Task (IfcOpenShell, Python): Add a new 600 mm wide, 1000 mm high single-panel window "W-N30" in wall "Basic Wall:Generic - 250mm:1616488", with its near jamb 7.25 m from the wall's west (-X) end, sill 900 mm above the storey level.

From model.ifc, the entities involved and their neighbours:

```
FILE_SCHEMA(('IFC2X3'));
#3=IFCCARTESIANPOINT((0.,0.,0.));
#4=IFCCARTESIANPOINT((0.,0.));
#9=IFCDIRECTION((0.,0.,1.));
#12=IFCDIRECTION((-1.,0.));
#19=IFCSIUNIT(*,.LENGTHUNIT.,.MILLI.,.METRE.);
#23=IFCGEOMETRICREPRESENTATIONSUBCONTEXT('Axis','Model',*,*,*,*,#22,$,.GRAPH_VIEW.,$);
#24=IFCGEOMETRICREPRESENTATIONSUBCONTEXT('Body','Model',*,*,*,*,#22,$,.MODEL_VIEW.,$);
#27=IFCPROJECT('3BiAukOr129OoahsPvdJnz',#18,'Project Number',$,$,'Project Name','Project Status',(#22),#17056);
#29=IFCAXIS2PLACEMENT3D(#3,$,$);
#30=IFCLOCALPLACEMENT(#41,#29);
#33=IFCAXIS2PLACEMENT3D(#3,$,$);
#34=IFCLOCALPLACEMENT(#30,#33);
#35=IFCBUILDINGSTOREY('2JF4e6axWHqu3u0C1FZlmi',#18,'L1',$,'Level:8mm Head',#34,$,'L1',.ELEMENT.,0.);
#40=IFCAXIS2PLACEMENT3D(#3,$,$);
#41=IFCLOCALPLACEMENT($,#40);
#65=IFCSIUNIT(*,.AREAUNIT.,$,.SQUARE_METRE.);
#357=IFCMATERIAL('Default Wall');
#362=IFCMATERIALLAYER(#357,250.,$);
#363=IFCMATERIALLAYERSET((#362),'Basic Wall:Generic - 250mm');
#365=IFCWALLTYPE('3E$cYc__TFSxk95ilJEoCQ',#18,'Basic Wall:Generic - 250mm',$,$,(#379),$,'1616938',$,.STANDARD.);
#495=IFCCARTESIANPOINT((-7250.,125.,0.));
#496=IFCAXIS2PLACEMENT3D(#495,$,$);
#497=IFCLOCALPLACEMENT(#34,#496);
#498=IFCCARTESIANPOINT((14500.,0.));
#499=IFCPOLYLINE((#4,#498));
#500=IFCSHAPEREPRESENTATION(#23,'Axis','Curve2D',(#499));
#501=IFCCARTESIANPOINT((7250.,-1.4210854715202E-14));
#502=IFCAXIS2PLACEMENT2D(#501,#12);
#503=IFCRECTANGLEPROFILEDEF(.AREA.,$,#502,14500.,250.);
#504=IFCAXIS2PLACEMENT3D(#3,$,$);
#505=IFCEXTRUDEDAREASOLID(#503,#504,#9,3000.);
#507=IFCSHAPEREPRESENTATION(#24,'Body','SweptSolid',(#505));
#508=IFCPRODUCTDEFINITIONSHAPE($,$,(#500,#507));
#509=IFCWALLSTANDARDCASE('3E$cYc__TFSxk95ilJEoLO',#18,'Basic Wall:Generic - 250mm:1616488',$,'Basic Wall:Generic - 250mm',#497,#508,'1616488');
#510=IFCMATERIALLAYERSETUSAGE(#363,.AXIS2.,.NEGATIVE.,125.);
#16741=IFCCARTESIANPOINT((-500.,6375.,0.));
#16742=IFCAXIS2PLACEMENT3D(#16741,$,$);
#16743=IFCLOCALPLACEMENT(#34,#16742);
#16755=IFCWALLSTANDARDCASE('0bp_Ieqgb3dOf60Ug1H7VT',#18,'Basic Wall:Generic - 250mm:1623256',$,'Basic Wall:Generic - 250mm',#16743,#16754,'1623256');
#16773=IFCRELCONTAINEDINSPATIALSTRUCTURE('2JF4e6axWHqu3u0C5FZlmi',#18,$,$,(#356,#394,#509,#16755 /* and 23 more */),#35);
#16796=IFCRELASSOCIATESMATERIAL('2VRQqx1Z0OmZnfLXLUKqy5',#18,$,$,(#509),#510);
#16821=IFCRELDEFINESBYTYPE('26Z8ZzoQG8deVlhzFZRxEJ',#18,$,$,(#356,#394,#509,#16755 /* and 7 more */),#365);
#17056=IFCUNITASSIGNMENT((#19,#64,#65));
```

```python
import numpy as np
import ifcopenshell
import ifcopenshell.api.feature
import ifcopenshell.api.geometry
import ifcopenshell.api.root
import ifcopenshell.api.spatial
import ifcopenshell.api.type
import ifcopenshell.geom
import ifcopenshell.util.element
import ifcopenshell.util.placement
import ifcopenshell.util.representation
import ifcopenshell.util.shape
import ifcopenshell.util.unit

model = ifcopenshell.open("model.ifc")
unit_scale = ifcopenshell.util.unit.calculate_unit_scale(model)
settings = ifcopenshell.geom.settings()


def volume(element):
    """Net volume in cubic metres, openings subtracted."""
    shape = ifcopenshell.geom.create_shape(settings, element)
    return ifcopenshell.util.shape.get_volume(shape.geometry)


wall = model.by_guid("3E$cYc__TFSxk95ilJEoLO")
storey = ifcopenshell.util.element.get_container(wall, ifc_class="IfcBuildingStorey")
context = ifcopenshell.util.representation.get_context(model, "Model", "Body", "MODEL_VIEW")
before = volume(wall)

width, height, from_end, sill = 0.6, 1, 7.25, 0.9  # metres

# The wall runs along its own X axis, and the end named is its -X end.
wall_shape = ifcopenshell.geom.create_shape(settings, wall)
x, y, z = ifcopenshell.util.shape.get_vertices(wall_shape.geometry).T
start = x.min() + from_end
face, thickness = float(y.min()), float(y.max() - y.min())
wall_matrix = ifcopenshell.util.placement.get_local_placement(wall.ObjectPlacement)
level = ifcopenshell.util.placement.get_local_placement(storey.ObjectPlacement)[2, 3]


def in_wall(x, y):
    """Placement at x, y metres in the wall's axes, at sill height."""
    matrix = wall_matrix.copy()
    matrix[:, 3] = wall_matrix @ np.array([x / unit_scale, y / unit_scale, 0.0, 1.0])
    matrix[2, 3] = level + sill / unit_scale
    return matrix


# Opening: a box that overshoots both wall faces by 50 mm.
opening = ifcopenshell.api.root.create_entity(model, ifc_class="IfcOpeningElement")
box = ifcopenshell.api.geometry.add_wall_representation(
    model, context=context, length=width, height=height, thickness=thickness + 0.1
)
ifcopenshell.api.geometry.assign_representation(model, product=opening, representation=box)
ifcopenshell.api.geometry.edit_object_placement(model, product=opening, matrix=in_wall(start, face - 0.05), is_si=False)
ifcopenshell.api.feature.add_feature(model, feature=opening, element=wall)

window = ifcopenshell.api.root.create_entity(model, ifc_class="IfcWindow", name="W-N30")
window.OverallWidth, window.OverallHeight = width / unit_scale, height / unit_scale
body = ifcopenshell.api.geometry.add_window_representation(
    model,
    context=context,
    overall_width=window.OverallWidth,
    overall_height=window.OverallHeight,
    partition_type="SINGLE_PANEL",
)
ifcopenshell.api.geometry.assign_representation(model, product=window, representation=body)
ifcopenshell.api.spatial.assign_container(model, products=[window], relating_structure=storey)
fills = ifcopenshell.api.feature.add_filling(model, opening=opening, element=window)
fills.OwnerHistory = window.OwnerHistory  # required in IFC2X3

# IFC2X3 keeps the operation on the window style.
style = ifcopenshell.api.root.create_entity(model, ifc_class="IfcWindowStyle", name="W-N30")
style.OperationType, style.ConstructionType = "SINGLE_PANEL", "NOTDEFINED"
style.ParameterTakesPrecedence = style.Sizeable = False
ifcopenshell.api.type.assign_type(model, related_objects=[window], relating_type=style)

# Centre the window in the wall's thickness.
ifcopenshell.api.geometry.edit_object_placement(model, product=window, matrix=in_wall(start, face), is_si=False)
window_shape = ifcopenshell.geom.create_shape(settings, window)
depth = ifcopenshell.util.shape.get_vertices(window_shape.geometry)[:, 1]
offset = face + thickness / 2 - (depth.min() + depth.max()) / 2
ifcopenshell.api.geometry.edit_object_placement(model, product=window, matrix=in_wall(start, offset), is_si=False)

after = volume(wall)

print(f"wall volume {before:.3f} -> {after:.3f} m3")

model.write("model_edited.ifc")
```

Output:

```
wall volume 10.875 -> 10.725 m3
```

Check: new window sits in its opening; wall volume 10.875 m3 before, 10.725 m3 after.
